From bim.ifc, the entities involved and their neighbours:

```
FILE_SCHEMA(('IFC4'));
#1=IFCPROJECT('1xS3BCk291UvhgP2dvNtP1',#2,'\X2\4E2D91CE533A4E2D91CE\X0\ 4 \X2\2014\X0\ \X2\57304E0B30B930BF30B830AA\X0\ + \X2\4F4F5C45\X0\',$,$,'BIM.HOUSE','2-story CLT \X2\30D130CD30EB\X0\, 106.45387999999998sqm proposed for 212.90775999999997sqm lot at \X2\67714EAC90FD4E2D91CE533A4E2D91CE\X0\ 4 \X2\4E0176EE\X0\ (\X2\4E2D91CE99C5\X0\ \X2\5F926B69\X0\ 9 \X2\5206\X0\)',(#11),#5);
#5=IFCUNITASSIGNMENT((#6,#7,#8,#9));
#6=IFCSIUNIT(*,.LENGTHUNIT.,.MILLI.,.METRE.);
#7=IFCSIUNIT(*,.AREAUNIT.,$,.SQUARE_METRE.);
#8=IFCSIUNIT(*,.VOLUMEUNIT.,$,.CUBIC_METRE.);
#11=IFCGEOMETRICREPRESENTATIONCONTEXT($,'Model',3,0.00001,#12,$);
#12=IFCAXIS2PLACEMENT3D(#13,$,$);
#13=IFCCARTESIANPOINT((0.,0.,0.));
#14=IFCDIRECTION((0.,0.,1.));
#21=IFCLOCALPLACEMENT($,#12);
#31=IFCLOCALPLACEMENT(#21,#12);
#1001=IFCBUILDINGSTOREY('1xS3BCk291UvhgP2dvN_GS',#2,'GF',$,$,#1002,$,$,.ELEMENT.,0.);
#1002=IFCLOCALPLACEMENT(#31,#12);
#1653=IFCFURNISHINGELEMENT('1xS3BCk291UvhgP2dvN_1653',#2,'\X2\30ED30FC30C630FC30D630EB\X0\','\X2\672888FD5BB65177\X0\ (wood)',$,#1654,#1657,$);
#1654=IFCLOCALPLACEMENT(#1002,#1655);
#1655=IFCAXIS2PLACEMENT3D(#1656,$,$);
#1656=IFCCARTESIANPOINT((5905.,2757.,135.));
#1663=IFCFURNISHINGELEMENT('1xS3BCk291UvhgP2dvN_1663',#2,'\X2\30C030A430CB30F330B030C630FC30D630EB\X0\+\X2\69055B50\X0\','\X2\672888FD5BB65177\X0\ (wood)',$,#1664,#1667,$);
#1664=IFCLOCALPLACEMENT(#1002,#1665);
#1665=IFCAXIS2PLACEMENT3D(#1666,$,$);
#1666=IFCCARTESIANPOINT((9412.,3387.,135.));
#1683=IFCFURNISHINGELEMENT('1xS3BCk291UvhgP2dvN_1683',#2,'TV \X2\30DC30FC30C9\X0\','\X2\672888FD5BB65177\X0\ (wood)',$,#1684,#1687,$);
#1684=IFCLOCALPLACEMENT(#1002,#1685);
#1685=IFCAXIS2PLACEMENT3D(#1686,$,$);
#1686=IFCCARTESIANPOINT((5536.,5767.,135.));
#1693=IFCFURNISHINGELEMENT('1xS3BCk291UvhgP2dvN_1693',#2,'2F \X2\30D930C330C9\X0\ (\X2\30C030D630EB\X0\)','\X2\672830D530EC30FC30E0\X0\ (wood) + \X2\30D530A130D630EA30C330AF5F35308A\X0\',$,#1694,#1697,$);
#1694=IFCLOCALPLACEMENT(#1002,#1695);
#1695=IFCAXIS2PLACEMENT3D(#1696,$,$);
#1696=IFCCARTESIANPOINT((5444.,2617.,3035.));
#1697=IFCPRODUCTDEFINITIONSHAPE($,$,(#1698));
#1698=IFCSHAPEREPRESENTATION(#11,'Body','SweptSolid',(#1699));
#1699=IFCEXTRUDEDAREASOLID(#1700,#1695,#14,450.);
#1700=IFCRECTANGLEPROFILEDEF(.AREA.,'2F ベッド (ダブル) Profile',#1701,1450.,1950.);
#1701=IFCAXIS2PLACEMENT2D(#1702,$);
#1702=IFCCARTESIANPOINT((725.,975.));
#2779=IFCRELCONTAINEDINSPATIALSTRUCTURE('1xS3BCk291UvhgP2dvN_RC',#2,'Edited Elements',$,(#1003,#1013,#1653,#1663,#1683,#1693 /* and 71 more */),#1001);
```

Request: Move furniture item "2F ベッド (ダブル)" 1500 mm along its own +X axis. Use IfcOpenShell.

```python
import ifcopenshell
import ifcopenshell.api.geometry
import ifcopenshell.util.placement

model = ifcopenshell.open("bim.ifc")

item = model.by_id(1693)
matrix = ifcopenshell.util.placement.get_local_placement(item.ObjectPlacement)
matrix[:3, 3] += matrix[:3, 0] * 1500.0
ifcopenshell.api.geometry.edit_object_placement(model, product=item, matrix=matrix, is_si=False)

print(ifcopenshell.util.placement.get_local_placement(item.ObjectPlacement).round(3) + 0.0)

model.write("bim_updated.ifc")
```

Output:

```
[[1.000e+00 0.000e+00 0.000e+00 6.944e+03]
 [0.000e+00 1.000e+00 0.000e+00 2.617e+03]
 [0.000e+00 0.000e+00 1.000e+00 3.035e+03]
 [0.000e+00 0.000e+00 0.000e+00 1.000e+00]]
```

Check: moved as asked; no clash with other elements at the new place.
